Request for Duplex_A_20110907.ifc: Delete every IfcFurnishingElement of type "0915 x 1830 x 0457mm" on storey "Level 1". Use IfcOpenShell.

First a look at what the model holds.

```python
import ifcopenshell
import ifcopenshell.util.element

model = ifcopenshell.open("Duplex_A_20110907.ifc")
print(model.schema)
storey = next(s for s in model.by_type("IfcBuildingStorey") if s.Name == "Level 1")
furniture = [e for e in ifcopenshell.util.element.get_decomposition(storey) if e.is_a("IfcFurnishingElement")]
seen = {}
for e in furniture:
    element_type = ifcopenshell.util.element.get_type(e)
    name = element_type.Name if element_type not in (None, e) else None
    seen[name] = seen.get(name, 0) + 1
for name, count in sorted(seen.items(), key=str):
    print(count, "x", name)
```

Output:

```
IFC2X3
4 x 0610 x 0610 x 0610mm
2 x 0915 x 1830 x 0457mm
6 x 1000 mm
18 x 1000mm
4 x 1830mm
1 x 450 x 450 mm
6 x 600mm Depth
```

```python
import ifcopenshell
import ifcopenshell.api.root
import ifcopenshell.util.element

model = ifcopenshell.open("Duplex_A_20110907.ifc")

storey = next(s for s in model.by_type("IfcBuildingStorey") if s.Name == "Level 1")
furniture = [e for e in ifcopenshell.util.element.get_decomposition(storey) if e.is_a("IfcFurnishingElement")]
targets = [e for e in furniture if (t := ifcopenshell.util.element.get_type(e)) not in (None, e) and t.Name == "0915 x 1830 x 0457mm"]

for e in targets:
    ifcopenshell.api.root.remove_product(model, product=e)
print(len(targets), "removed")

model.write("Duplex_A_20110907_updated.ifc")
```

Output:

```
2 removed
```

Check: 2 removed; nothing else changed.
